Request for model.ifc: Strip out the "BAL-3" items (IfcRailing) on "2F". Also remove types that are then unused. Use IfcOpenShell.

First a look at what the model holds.

```python
import ifcopenshell
import ifcopenshell.util.element

model = ifcopenshell.open("model.ifc")
print(model.schema)
storey = next(s for s in model.by_type("IfcBuildingStorey") if s.Name == "2F")
railings = [e for e in ifcopenshell.util.element.get_decomposition(storey) if e.is_a("IfcRailing")]
seen = {}
for e in railings:
    element_type = ifcopenshell.util.element.get_type(e)
    name = element_type.Name if element_type not in (None, e) else None
    seen[name] = seen.get(name, 0) + 1
for name, count in sorted(seen.items(), key=str):
    print(count, "x", name)
```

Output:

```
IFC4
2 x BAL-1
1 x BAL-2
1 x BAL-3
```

```python
import ifcopenshell
import ifcopenshell.api.root
import ifcopenshell.util.element

model = ifcopenshell.open("model.ifc")

storey = next(s for s in model.by_type("IfcBuildingStorey") if s.Name == "2F")
railings = [e for e in ifcopenshell.util.element.get_decomposition(storey) if e.is_a("IfcRailing")]
targets = [e for e in railings if (t := ifcopenshell.util.element.get_type(e)) not in (None, e) and t.Name == "BAL-3"]
types = {ifcopenshell.util.element.get_type(e) for e in targets} - {None, *targets}

for e in targets:
    ifcopenshell.api.root.remove_product(model, product=e)
print(len(targets), "removed")

unused = [t for t in types if not ifcopenshell.util.element.get_types(t)]
for t in unused:
    ifcopenshell.api.root.remove_product(model, product=t)
print(len(unused), "unused types removed")

model.write("model_v2.ifc")
```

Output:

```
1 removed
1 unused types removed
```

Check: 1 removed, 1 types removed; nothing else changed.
